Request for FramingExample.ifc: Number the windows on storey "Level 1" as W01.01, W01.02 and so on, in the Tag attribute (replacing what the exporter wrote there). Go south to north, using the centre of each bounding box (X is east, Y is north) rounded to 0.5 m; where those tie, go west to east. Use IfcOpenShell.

First a look at what the model holds.

```python
import ifcopenshell
import ifcopenshell.util.element
import ifcopenshell.util.placement

model = ifcopenshell.open("FramingExample.ifc")
print(model.schema)
storey = next(s for s in model.by_type("IfcBuildingStorey") if s.Name == "Level 1")
windows = [e for e in ifcopenshell.util.element.get_decomposition(storey) if e.is_a("IfcWindow")]
for e in sorted(windows, key=lambda e: e.id()):
    origin = ifcopenshell.util.placement.get_local_placement(e.ObjectPlacement)[:3, 3]
    print(e.id(), e.Tag, e.Name, origin.round(2) + 0.0, sep=" | ")
```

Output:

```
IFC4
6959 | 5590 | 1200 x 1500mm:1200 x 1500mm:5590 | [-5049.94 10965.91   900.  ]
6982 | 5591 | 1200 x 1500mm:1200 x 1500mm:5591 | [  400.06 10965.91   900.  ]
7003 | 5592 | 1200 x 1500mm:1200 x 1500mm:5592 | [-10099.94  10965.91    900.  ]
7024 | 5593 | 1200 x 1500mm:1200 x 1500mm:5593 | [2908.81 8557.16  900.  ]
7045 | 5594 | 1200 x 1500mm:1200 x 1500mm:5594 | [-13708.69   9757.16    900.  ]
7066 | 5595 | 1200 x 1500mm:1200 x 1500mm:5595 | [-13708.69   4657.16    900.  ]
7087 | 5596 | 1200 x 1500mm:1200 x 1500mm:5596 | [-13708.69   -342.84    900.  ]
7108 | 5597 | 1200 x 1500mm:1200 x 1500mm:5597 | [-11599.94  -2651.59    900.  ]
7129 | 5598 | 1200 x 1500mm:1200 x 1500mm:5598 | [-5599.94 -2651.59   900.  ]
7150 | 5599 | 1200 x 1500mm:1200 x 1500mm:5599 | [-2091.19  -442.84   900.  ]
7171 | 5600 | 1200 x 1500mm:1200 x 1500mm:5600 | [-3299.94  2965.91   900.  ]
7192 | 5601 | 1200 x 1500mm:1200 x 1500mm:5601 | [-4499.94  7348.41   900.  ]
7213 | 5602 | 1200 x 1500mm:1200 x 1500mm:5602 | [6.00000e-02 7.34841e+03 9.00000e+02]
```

```python
import ifcopenshell
import ifcopenshell.geom
import ifcopenshell.util.element
import ifcopenshell.util.shape

model = ifcopenshell.open("FramingExample.ifc")
settings = ifcopenshell.geom.settings()
settings.set("use-world-coords", True)


def centre(element):
    shape = ifcopenshell.geom.create_shape(settings, element)
    return ifcopenshell.util.shape.get_bbox_centroid(shape.geometry)


storey = next(s for s in model.by_type("IfcBuildingStorey") if s.Name == "Level 1")
windows = [e for e in ifcopenshell.util.element.get_decomposition(storey) if e.is_a("IfcWindow")]

# Insertion points can sit at a corner or the storey origin, so sort by the geometry (in metres).
centres = {e: centre(e) for e in windows}
windows.sort(key=lambda e: (round(centres[e][1] / 0.5), centres[e][0]))

for i, e in enumerate(windows, start=1):
    number = f"W01.{i:02d}"
    e.Tag = number
    print(e.id(), number)

model.write("FramingExample_rev.ifc")
```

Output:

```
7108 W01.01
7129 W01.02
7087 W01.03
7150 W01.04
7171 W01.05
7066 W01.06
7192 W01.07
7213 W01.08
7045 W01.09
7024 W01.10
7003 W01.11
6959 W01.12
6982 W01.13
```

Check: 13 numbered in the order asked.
